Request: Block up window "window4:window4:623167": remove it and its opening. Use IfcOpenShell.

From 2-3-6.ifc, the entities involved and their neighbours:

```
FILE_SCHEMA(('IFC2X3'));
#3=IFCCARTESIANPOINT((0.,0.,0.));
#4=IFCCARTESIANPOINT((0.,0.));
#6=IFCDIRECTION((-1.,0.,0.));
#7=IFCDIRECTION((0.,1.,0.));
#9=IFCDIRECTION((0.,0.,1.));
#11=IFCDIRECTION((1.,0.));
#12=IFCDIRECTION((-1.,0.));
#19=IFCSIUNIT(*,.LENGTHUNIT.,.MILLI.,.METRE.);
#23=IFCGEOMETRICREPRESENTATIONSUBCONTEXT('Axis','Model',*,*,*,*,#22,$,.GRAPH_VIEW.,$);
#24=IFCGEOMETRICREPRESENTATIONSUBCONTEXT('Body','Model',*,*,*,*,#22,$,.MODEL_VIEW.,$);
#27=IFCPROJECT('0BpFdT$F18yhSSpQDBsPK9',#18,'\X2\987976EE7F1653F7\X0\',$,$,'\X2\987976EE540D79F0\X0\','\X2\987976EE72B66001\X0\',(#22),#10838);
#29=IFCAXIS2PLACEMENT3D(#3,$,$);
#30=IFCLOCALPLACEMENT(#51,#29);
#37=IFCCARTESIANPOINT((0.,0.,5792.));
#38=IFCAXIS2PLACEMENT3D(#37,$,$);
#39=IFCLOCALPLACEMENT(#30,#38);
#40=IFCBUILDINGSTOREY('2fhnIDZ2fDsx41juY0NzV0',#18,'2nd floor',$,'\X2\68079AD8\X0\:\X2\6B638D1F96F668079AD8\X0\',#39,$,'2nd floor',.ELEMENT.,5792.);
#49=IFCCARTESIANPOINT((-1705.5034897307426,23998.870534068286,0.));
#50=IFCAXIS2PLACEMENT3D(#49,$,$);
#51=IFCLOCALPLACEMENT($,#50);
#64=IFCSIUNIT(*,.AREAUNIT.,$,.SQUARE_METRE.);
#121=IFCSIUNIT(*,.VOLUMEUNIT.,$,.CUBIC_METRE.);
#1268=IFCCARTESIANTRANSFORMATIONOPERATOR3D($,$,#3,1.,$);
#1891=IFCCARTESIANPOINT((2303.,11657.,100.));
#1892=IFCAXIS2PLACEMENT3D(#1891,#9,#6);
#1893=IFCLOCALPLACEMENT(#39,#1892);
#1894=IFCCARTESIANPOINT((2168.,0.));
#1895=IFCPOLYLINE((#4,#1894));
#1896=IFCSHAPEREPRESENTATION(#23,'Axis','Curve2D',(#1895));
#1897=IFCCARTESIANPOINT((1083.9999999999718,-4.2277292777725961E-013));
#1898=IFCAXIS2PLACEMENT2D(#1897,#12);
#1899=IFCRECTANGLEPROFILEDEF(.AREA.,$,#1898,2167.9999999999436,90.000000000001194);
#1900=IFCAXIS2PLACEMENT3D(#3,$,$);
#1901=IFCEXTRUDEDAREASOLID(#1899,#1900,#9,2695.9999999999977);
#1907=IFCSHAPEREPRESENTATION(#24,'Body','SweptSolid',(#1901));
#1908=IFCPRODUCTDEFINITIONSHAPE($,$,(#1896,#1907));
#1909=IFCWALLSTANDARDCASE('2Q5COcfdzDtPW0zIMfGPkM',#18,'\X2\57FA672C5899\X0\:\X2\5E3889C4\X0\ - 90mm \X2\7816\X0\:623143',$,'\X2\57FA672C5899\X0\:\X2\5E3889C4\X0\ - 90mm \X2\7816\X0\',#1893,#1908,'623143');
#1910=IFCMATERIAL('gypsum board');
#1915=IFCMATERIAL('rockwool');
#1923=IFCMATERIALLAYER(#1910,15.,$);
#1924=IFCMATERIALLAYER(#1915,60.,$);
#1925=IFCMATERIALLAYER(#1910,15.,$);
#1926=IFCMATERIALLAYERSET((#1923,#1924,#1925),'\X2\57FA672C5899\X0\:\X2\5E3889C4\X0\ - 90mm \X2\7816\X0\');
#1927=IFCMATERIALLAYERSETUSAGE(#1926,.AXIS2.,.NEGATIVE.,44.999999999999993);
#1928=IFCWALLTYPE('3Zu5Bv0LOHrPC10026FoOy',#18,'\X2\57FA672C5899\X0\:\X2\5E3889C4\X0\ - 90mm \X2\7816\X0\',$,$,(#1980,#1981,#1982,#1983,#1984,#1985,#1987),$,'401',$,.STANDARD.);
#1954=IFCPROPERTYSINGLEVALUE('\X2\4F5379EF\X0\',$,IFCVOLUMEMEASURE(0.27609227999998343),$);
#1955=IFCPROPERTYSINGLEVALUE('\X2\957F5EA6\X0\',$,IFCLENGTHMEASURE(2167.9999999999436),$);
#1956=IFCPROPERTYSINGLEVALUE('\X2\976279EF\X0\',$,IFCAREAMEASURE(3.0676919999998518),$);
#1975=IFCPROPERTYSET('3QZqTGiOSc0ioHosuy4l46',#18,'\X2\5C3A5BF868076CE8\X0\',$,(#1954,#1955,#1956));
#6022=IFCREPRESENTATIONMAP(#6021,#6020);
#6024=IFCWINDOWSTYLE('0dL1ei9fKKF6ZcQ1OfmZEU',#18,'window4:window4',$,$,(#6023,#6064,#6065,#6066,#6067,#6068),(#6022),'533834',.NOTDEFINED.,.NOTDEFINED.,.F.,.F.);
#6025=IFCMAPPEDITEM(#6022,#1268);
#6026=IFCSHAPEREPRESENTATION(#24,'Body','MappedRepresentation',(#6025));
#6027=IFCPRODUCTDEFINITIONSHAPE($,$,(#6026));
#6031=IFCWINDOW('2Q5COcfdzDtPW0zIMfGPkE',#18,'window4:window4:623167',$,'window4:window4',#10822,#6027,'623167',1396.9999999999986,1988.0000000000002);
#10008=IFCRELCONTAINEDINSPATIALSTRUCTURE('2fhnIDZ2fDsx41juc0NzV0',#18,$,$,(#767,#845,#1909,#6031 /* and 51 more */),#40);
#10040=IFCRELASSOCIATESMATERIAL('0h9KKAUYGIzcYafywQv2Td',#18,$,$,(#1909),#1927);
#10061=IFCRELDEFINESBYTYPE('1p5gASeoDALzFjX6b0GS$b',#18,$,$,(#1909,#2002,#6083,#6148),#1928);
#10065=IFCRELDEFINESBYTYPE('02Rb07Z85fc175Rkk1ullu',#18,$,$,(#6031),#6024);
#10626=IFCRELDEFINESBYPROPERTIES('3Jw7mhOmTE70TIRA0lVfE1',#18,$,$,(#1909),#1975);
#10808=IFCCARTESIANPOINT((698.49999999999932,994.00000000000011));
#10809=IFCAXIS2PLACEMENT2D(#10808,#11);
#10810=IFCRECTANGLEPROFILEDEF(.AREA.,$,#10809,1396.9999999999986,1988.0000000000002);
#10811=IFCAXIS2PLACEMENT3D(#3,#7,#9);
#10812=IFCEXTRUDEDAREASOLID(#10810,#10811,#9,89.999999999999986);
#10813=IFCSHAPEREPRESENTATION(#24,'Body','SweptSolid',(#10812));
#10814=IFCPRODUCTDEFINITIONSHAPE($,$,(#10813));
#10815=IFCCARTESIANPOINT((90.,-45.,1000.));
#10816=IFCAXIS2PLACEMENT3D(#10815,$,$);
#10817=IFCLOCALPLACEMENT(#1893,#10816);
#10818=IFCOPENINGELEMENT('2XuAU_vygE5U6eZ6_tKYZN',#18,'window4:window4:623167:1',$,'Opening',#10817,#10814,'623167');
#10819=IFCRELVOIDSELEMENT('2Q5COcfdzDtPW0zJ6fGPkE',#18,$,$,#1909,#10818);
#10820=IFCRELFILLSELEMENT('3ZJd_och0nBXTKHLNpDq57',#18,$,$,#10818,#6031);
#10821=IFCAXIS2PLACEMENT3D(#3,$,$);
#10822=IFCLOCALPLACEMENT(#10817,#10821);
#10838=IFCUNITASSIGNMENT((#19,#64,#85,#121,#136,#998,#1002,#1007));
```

```python
import ifcopenshell
import ifcopenshell.api.feature
import ifcopenshell.api.pset
import ifcopenshell.api.root
import ifcopenshell.geom
import ifcopenshell.util.element
import ifcopenshell.util.shape
import ifcopenshell.util.unit

model = ifcopenshell.open("2-3-6.ifc")
area_scale = ifcopenshell.util.unit.calculate_unit_scale(model, "AREAUNIT")
volume_scale = ifcopenshell.util.unit.calculate_unit_scale(model, "VOLUMEUNIT")
settings = ifcopenshell.geom.settings()


def volume(element):
    """Net volume in cubic metres, openings subtracted."""
    shape = ifcopenshell.geom.create_shape(settings, element)
    return ifcopenshell.util.shape.get_volume(shape.geometry)


window = model.by_guid("2Q5COcfdzDtPW0zIMfGPkE")
opening = window.FillsVoids[0].RelatingOpeningElement
wall = opening.VoidsElements[0].RelatingBuildingElement
before = volume(wall)

ifcopenshell.api.root.remove_product(model, product=window)
ifcopenshell.api.feature.remove_feature(model, feature=opening)

after = volume(wall)
thickness = 0.09  # wall thickness in metres

# Update the wall's stored quantities.
pset = model.by_id(ifcopenshell.util.element.get_pset(wall, "尺寸标注", should_inherit=False)["id"])
ifcopenshell.api.pset.edit_pset(model, pset=pset, properties={
    "体积": model.create_entity("IfcVolumeMeasure", after / volume_scale),
    "面积": model.create_entity("IfcAreaMeasure", after / thickness / area_scale),
})

print(f"wall volume {before:.3f} -> {after:.3f} m3")

model.write("2-3-6_updated.ifc")
```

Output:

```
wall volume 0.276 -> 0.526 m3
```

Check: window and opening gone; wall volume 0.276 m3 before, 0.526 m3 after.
